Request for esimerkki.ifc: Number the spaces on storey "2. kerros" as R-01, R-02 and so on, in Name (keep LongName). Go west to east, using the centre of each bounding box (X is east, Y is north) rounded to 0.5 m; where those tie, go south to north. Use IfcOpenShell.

First a look at what the model holds.

```python
import ifcopenshell
import ifcopenshell.util.element
import ifcopenshell.util.placement

model = ifcopenshell.open("esimerkki.ifc")
print(model.schema)
storey = next(s for s in model.by_type("IfcBuildingStorey") if s.Name == "2. kerros")
spaces = [e for e in ifcopenshell.util.element.get_decomposition(storey) if e.is_a("IfcSpace")]
for e in sorted(spaces, key=lambda e: e.id()):
    origin = ifcopenshell.util.placement.get_local_placement(e.ObjectPlacement)[:3, 3]
    print(e.id(), e.Name, e.LongName, origin.round(2) + 0.0, sep=" | ")
```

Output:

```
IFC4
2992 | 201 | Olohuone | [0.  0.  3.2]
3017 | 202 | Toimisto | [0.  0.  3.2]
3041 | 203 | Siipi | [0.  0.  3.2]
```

```python
import ifcopenshell
import ifcopenshell.geom
import ifcopenshell.util.element
import ifcopenshell.util.shape

model = ifcopenshell.open("esimerkki.ifc")
settings = ifcopenshell.geom.settings()
settings.set("use-world-coords", True)


def centre(element):
    shape = ifcopenshell.geom.create_shape(settings, element)
    return ifcopenshell.util.shape.get_bbox_centroid(shape.geometry)


storey = next(s for s in model.by_type("IfcBuildingStorey") if s.Name == "2. kerros")
spaces = [e for e in ifcopenshell.util.element.get_decomposition(storey) if e.is_a("IfcSpace")]

# Insertion points can sit at a corner or the storey origin, so sort by the geometry (in metres).
centres = {e: centre(e) for e in spaces}
spaces.sort(key=lambda e: (round(centres[e][0] / 0.5), centres[e][1]))

for i, e in enumerate(spaces, start=1):
    number = f"R-{i:02d}"
    e.Name = number
    print(e.id(), number)

model.write("esimerkki-out.ifc")
```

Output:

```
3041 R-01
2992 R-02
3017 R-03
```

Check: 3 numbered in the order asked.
